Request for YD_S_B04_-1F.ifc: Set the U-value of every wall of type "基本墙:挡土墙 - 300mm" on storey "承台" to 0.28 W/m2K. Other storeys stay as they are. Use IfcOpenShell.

First a look at what the model holds.

```python
import ifcopenshell
import ifcopenshell.util.element

model = ifcopenshell.open("YD_S_B04_-1F.ifc")
print(model.schema)
storey = next(s for s in model.by_type("IfcBuildingStorey") if s.Name == "承台")
walls = [e for e in ifcopenshell.util.element.get_decomposition(storey) if e.is_a("IfcWall")]
seen = {}
for e in walls:
    element_type = ifcopenshell.util.element.get_type(e)
    key = (element_type.Name if element_type != e and element_type else None, ifcopenshell.util.element.get_pset(e, "Pset_WallCommon", "ThermalTransmittance"))
    seen[key] = seen.get(key, 0) + 1
for (name, value), count in sorted(seen.items(), key=str):
    print(count, "x", name, "|", value)
```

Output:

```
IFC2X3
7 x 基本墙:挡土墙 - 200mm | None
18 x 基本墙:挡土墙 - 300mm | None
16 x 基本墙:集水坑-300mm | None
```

```python
import ifcopenshell
import ifcopenshell.api.pset
import ifcopenshell.util.element

model = ifcopenshell.open("YD_S_B04_-1F.ifc")

storey = next(s for s in model.by_type("IfcBuildingStorey") if s.Name == "承台")
walls = [e for e in ifcopenshell.util.element.get_decomposition(storey) if e.is_a("IfcWall")]

count = 0
for e in walls:
    element_type = ifcopenshell.util.element.get_type(e)
    if element_type in (None, e) or element_type.Name != "基本墙:挡土墙 - 300mm":
        continue
    # add_pset returns the element's existing set when there is one.
    pset = ifcopenshell.api.pset.add_pset(model, product=e, name="Pset_WallCommon")
    ifcopenshell.api.pset.edit_pset(model, pset=pset, properties={"ThermalTransmittance": 0.28})
    count += 1

print(count, "walls updated")

model.write("YD_S_B04_-1F_updated.ifc")
```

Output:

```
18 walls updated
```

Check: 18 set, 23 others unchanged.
